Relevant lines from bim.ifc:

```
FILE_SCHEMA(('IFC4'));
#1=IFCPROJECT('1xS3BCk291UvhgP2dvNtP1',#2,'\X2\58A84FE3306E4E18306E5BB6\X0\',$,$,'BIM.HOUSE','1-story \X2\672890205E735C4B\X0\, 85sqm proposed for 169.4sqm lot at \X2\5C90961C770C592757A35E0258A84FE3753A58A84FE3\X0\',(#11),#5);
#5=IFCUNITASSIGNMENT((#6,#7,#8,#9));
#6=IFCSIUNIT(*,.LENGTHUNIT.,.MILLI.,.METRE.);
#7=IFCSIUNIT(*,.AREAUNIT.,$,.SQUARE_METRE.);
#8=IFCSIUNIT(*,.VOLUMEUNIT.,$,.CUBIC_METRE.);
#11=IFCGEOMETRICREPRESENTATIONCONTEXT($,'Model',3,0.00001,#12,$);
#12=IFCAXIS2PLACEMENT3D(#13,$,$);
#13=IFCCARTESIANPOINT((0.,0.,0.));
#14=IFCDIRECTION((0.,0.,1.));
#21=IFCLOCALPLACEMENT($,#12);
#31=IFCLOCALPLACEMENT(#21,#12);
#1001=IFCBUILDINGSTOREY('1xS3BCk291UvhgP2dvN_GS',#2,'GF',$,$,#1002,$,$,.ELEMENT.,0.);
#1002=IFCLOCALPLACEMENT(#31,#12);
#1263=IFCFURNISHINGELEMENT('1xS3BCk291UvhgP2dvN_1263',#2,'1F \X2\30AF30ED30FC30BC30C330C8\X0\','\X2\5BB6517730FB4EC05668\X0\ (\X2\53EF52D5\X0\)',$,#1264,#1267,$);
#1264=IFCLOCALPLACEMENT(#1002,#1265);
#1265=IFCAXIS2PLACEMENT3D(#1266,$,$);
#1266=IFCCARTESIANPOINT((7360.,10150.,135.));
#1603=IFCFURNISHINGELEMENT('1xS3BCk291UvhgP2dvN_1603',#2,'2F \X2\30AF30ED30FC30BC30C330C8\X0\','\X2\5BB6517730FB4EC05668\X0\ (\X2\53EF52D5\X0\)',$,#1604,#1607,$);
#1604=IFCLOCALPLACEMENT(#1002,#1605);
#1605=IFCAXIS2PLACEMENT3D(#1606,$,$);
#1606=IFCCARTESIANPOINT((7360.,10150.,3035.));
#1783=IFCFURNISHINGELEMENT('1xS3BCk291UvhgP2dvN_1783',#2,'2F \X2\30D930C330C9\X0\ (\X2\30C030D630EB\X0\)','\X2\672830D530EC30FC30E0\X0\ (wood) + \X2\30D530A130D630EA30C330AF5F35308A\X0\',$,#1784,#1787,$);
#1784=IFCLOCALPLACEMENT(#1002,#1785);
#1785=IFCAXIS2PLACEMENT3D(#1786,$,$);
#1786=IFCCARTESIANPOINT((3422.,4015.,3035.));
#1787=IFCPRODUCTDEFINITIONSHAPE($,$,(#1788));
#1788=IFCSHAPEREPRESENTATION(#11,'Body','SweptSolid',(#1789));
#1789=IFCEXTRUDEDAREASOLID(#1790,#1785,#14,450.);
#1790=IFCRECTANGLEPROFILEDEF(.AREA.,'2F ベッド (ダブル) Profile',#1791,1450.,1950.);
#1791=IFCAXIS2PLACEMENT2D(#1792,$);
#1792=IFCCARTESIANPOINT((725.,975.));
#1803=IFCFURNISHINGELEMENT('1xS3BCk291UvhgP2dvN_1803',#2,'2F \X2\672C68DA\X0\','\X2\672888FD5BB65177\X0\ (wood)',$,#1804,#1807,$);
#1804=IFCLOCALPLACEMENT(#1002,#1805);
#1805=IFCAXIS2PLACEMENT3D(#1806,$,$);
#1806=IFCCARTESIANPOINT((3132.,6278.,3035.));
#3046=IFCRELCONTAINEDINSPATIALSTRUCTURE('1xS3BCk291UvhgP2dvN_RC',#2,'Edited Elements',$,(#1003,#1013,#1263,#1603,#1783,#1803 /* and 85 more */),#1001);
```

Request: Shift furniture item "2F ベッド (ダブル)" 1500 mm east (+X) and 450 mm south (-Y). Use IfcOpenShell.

```python
import ifcopenshell
import ifcopenshell.api.geometry
import ifcopenshell.util.placement
import ifcopenshell.util.unit

model = ifcopenshell.open("bim.ifc")
unit_scale = ifcopenshell.util.unit.calculate_unit_scale(model)

item = model.by_guid("1xS3BCk291UvhgP2dvN_1783")
matrix = ifcopenshell.util.placement.get_local_placement(item.ObjectPlacement)
matrix[0, 3] += 1.5 / unit_scale
matrix[1, 3] -= 0.45 / unit_scale
ifcopenshell.api.geometry.edit_object_placement(model, product=item, matrix=matrix, is_si=False)

print(ifcopenshell.util.placement.get_local_placement(item.ObjectPlacement).round(3) + 0.0)

model.write("bim_v2.ifc")
```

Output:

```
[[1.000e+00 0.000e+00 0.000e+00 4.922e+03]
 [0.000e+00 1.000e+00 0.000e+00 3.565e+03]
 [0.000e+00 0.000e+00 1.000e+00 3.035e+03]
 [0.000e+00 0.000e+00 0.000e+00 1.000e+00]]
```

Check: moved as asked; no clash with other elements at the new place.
